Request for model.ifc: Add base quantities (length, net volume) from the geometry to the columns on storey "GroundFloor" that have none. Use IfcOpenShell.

First a look at what the model holds.

```python
import ifcopenshell
import ifcopenshell.util.element
import ifcopenshell.util.unit

model = ifcopenshell.open("model.ifc")
print(model.schema)
for unit_type in ("LENGTHUNIT", "AREAUNIT", "VOLUMEUNIT"):
    print(unit_type, ifcopenshell.util.unit.calculate_unit_scale(model, unit_type))
storey = next(s for s in model.by_type("IfcBuildingStorey") if s.Name == "GroundFloor")
columns = [e for e in ifcopenshell.util.element.get_decomposition(storey) if e.is_a("IfcColumn")]
for e in sorted(columns, key=lambda e: e.id()):
    print(e.id(), e.is_a(), e.Name, list(ifcopenshell.util.element.get_psets(e, qtos_only=True)), sep=" | ")
```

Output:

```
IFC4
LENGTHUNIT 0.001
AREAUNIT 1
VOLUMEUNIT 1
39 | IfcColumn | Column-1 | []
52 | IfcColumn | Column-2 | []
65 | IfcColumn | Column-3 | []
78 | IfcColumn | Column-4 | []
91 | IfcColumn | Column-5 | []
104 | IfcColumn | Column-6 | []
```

```python
import ifcopenshell
import ifcopenshell.api.pset
import ifcopenshell.geom
import ifcopenshell.util.element
import ifcopenshell.util.shape
import ifcopenshell.util.unit

model = ifcopenshell.open("model.ifc")
unit_scale = ifcopenshell.util.unit.calculate_unit_scale(model)
volume_scale = ifcopenshell.util.unit.calculate_unit_scale(model, "VOLUMEUNIT")
settings = ifcopenshell.geom.settings()

storey = next(s for s in model.by_type("IfcBuildingStorey") if s.Name == "GroundFloor")
columns = [e for e in ifcopenshell.util.element.get_decomposition(storey) if e.is_a("IfcColumn")]

for e in sorted(columns, key=lambda e: e.id()):
    if ifcopenshell.util.element.get_psets(e, qtos_only=True, should_inherit=False):
        continue
    # Geometry comes back in metres, in the element's own axes.
    shape = ifcopenshell.geom.create_shape(settings, e)
    values = {
        "Length": ifcopenshell.util.shape.get_z(shape.geometry) / unit_scale,
        "NetVolume": ifcopenshell.util.shape.get_volume(shape.geometry) / volume_scale,
    }
    qto = ifcopenshell.api.pset.add_qto(model, product=e, name="Qto_ColumnBaseQuantities")
    ifcopenshell.api.pset.edit_qto(model, qto=qto, properties=values)
    print(e.id(), {k: round(v, 3) for k, v in values.items()})

model.write("model_edited.ifc")
```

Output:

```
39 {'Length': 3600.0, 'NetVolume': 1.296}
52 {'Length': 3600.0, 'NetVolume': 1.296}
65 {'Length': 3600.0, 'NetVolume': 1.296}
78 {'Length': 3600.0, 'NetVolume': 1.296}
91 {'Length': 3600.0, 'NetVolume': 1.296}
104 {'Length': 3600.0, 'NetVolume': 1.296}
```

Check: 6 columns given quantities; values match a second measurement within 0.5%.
